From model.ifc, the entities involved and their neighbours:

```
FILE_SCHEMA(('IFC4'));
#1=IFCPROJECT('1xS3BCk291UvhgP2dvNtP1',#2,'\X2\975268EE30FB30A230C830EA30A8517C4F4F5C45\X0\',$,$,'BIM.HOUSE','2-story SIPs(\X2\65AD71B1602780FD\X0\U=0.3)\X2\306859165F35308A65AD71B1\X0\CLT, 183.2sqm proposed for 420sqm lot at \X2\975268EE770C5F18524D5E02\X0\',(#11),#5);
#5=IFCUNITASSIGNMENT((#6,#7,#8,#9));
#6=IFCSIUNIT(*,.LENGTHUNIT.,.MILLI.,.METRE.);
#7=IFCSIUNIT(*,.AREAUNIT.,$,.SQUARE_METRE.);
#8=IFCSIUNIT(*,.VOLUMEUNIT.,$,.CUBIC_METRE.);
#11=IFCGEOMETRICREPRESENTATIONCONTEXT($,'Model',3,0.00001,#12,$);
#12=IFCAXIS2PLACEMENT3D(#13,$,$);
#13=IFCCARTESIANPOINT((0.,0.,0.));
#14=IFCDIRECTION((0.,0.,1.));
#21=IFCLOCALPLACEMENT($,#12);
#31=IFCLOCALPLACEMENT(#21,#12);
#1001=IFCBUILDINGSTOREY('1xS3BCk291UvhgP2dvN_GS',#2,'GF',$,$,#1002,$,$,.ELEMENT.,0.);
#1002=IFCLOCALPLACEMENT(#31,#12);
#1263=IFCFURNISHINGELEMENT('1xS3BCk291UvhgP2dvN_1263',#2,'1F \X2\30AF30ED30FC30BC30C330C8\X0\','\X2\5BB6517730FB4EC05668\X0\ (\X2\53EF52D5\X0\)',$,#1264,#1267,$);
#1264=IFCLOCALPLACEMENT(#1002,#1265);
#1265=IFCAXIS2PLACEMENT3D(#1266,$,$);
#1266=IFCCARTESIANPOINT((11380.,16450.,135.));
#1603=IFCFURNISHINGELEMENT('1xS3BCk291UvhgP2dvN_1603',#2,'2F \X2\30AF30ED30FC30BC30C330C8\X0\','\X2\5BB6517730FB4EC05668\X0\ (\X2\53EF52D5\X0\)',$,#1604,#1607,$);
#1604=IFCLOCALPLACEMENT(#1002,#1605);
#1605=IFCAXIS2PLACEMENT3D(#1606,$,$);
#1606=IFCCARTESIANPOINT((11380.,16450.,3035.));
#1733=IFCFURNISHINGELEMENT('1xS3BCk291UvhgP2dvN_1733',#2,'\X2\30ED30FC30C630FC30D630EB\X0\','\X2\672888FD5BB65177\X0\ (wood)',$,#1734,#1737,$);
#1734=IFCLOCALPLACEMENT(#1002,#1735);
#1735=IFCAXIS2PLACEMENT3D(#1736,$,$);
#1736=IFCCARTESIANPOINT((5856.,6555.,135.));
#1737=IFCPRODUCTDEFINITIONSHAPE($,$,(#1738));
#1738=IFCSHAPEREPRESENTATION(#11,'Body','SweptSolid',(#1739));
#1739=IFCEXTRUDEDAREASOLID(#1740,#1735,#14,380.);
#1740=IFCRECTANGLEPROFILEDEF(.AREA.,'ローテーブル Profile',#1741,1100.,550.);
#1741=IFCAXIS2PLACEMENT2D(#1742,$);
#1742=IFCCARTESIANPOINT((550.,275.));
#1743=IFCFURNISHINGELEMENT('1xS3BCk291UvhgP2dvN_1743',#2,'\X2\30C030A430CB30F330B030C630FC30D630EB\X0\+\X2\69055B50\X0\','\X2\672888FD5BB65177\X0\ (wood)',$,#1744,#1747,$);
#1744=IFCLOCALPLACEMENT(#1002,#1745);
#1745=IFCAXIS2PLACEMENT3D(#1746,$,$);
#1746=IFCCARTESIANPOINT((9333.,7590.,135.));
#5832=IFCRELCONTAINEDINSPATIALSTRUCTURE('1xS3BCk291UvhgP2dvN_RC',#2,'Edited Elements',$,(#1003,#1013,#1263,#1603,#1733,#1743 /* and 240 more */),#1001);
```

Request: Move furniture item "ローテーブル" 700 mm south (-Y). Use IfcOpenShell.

```python
import ifcopenshell
import ifcopenshell.api.geometry
import ifcopenshell.util.placement

model = ifcopenshell.open("model.ifc")

item = model.by_guid("1xS3BCk291UvhgP2dvN_1733")
matrix = ifcopenshell.util.placement.get_local_placement(item.ObjectPlacement)
matrix[1, 3] -= 700.0
ifcopenshell.api.geometry.edit_object_placement(model, product=item, matrix=matrix, is_si=False)

print(ifcopenshell.util.placement.get_local_placement(item.ObjectPlacement).round(3) + 0.0)

model.write("model-out.ifc")
```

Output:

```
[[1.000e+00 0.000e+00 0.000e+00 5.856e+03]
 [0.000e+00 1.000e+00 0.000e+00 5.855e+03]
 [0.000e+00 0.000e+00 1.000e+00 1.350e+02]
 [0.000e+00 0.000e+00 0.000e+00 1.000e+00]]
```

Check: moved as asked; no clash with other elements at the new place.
